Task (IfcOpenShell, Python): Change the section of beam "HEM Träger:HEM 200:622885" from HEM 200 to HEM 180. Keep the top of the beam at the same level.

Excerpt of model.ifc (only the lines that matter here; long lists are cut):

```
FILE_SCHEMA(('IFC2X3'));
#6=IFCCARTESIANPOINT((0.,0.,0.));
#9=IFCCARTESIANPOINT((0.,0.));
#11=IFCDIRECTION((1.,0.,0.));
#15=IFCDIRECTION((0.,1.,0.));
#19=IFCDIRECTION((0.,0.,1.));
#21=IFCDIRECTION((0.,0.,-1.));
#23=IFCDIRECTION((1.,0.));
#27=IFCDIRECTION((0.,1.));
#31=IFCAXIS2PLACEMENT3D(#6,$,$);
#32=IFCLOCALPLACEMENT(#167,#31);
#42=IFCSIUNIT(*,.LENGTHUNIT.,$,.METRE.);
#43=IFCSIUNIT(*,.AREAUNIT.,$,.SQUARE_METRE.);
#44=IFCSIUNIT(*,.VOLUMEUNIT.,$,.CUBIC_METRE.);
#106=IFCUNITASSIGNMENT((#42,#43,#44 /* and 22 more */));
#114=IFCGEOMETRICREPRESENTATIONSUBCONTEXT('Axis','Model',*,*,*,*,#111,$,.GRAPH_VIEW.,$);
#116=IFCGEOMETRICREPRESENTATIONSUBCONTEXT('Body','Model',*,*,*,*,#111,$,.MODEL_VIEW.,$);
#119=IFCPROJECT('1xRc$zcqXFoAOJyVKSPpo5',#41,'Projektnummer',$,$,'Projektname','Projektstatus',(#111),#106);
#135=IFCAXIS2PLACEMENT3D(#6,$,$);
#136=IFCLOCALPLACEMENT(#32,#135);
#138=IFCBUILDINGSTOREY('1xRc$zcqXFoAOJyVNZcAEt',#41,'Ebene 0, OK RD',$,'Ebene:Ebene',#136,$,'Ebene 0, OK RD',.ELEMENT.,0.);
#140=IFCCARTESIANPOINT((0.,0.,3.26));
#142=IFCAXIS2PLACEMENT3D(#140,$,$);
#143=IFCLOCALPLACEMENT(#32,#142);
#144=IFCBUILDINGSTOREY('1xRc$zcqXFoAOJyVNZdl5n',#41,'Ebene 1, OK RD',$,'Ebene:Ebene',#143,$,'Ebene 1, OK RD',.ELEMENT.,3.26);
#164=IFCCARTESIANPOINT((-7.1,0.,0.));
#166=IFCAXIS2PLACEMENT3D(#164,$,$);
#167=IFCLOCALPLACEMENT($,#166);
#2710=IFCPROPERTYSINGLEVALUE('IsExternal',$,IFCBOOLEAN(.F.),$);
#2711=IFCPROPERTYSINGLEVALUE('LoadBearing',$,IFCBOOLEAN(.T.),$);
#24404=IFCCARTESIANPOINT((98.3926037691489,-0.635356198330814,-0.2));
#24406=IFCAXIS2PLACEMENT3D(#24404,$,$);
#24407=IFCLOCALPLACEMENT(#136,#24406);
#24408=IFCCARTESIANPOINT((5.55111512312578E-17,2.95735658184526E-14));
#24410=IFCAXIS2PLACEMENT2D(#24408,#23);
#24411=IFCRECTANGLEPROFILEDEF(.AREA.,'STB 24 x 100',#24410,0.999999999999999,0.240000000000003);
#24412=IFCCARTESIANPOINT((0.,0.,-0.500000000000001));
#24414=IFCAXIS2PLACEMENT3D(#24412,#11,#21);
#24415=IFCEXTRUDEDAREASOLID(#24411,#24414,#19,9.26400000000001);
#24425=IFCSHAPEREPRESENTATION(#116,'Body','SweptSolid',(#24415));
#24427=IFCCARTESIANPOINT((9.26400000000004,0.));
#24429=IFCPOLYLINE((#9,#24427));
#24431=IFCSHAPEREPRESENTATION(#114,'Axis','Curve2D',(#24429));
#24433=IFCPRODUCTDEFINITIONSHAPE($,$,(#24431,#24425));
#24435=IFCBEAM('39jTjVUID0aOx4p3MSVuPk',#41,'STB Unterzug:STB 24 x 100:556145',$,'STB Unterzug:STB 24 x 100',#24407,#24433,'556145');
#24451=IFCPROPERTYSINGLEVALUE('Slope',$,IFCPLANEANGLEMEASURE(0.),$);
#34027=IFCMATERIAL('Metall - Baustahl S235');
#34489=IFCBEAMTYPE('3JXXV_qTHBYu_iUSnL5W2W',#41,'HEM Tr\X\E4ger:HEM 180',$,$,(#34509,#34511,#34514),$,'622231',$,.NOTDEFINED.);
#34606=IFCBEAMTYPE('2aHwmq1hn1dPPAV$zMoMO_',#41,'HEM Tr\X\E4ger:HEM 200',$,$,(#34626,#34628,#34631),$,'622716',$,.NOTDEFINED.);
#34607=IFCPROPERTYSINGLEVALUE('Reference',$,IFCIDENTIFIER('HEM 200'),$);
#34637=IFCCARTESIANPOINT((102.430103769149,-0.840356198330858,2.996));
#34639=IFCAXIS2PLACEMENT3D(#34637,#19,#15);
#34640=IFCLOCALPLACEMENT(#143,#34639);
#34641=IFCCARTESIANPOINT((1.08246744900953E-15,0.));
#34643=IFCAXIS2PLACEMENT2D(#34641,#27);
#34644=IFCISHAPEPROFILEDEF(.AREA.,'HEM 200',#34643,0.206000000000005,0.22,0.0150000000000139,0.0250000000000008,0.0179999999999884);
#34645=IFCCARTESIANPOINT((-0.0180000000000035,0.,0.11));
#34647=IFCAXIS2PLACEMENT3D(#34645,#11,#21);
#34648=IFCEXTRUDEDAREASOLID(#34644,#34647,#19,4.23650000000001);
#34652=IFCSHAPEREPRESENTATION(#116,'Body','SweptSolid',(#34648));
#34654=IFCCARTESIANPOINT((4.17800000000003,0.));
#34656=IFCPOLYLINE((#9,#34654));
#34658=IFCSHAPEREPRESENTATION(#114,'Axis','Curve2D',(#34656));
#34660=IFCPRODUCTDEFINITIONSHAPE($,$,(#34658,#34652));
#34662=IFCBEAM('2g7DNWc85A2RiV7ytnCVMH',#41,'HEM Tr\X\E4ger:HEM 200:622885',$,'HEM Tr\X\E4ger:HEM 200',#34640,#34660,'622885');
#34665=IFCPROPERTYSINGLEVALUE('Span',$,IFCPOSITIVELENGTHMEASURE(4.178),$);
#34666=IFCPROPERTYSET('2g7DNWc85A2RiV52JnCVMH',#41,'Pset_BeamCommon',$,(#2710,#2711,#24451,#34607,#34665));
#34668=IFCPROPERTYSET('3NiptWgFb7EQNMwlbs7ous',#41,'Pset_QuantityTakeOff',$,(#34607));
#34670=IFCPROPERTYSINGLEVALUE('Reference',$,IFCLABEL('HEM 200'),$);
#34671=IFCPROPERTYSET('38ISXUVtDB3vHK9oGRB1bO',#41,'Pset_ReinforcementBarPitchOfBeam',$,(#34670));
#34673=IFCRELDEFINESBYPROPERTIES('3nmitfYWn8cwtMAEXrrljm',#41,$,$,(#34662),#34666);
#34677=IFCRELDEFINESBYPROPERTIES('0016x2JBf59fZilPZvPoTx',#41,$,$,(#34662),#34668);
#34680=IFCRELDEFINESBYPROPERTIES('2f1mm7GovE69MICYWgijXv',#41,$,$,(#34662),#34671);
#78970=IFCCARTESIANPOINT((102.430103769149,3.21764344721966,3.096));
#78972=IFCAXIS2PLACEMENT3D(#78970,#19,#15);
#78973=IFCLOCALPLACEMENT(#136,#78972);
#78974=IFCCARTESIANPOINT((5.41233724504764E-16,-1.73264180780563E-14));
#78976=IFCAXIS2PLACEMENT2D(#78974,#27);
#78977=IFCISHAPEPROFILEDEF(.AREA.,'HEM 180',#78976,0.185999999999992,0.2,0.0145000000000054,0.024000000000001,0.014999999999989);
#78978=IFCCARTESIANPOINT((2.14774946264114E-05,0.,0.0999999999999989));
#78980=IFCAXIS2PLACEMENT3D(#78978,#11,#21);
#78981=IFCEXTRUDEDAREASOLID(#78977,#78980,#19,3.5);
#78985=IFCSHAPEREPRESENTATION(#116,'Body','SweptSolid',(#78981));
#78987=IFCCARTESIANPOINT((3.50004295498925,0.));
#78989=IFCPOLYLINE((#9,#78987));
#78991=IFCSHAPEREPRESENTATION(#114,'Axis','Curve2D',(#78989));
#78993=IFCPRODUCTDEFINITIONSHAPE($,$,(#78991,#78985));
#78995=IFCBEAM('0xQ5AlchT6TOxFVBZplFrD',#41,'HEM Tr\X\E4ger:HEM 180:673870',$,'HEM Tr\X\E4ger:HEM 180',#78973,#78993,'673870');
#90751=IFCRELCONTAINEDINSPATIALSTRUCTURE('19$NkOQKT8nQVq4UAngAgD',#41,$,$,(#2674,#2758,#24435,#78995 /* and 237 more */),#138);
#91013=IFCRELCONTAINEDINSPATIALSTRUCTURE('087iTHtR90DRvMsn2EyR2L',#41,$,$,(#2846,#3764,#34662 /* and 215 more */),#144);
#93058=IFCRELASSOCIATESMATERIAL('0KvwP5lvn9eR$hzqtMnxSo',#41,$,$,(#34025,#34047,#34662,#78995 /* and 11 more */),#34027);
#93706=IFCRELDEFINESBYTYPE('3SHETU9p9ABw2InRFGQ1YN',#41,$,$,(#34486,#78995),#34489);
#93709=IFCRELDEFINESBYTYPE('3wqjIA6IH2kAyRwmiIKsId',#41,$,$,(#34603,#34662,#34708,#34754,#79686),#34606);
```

```python
import ifcopenshell
import ifcopenshell.api.pset
import ifcopenshell.api.type
import ifcopenshell.util.element
import ifcopenshell.util.representation

model = ifcopenshell.open("model.ifc")

member = model.by_id(34662)
source = next(p for p in model.by_type("IfcIShapeProfileDef") if p.ProfileName == "HEM 180")

body = ifcopenshell.util.representation.get_representation(member, "Model", "Body")
solid = body.Items[0]
old_profile = solid.SweptArea

# Copy the section's sizes but keep this member's own profile position.
profile = ifcopenshell.util.element.copy(model, source)
# Profiles are centred, so shift by half the change in depth to hold the top.
shift = (old_profile.OverallDepth - profile.OverallDepth) / 2
x, y = old_profile.Position.Location.Coordinates
up = (-1.0, 0.0)  # upwards, in the solid's own plane
location = model.createIfcCartesianPoint((x + up[0] * shift, y + up[1] * shift))
profile.Position = model.createIfcAxis2Placement2D(location, old_profile.Position.RefDirection)
solid.SweptArea = profile
if not model.get_total_inverses(old_profile):
    ifcopenshell.util.element.remove_deep2(model, old_profile)

new_type = model.by_guid("3JXXV_qTHBYu_iUSnL5W2W")
ifcopenshell.api.type.assign_type(
    model, related_objects=[member], relating_type=new_type, should_map_representations=False
)
member.Name = member.Name.replace("HEM 200", "HEM 180")
member.ObjectType = "HEM Träger:HEM 180"
pset = model.by_id(ifcopenshell.util.element.get_pset(member, "Pset_BeamCommon", should_inherit=False)["id"])
ifcopenshell.api.pset.edit_pset(model, pset=pset, properties={"Reference": "HEM 180"})
pset = model.by_id(ifcopenshell.util.element.get_pset(member, "Pset_QuantityTakeOff", should_inherit=False)["id"])
ifcopenshell.api.pset.edit_pset(model, pset=pset, properties={"Reference": "HEM 180"})
pset = model.by_id(ifcopenshell.util.element.get_pset(member, "Pset_ReinforcementBarPitchOfBeam", should_inherit=False)["id"])
ifcopenshell.api.pset.edit_pset(model, pset=pset, properties={"Reference": "HEM 180"})

print(solid.SweptArea)

model.write("model_rev.ifc")
```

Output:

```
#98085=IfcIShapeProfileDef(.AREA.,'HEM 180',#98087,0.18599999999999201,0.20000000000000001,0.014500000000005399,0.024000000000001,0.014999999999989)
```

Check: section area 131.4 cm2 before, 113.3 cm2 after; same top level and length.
